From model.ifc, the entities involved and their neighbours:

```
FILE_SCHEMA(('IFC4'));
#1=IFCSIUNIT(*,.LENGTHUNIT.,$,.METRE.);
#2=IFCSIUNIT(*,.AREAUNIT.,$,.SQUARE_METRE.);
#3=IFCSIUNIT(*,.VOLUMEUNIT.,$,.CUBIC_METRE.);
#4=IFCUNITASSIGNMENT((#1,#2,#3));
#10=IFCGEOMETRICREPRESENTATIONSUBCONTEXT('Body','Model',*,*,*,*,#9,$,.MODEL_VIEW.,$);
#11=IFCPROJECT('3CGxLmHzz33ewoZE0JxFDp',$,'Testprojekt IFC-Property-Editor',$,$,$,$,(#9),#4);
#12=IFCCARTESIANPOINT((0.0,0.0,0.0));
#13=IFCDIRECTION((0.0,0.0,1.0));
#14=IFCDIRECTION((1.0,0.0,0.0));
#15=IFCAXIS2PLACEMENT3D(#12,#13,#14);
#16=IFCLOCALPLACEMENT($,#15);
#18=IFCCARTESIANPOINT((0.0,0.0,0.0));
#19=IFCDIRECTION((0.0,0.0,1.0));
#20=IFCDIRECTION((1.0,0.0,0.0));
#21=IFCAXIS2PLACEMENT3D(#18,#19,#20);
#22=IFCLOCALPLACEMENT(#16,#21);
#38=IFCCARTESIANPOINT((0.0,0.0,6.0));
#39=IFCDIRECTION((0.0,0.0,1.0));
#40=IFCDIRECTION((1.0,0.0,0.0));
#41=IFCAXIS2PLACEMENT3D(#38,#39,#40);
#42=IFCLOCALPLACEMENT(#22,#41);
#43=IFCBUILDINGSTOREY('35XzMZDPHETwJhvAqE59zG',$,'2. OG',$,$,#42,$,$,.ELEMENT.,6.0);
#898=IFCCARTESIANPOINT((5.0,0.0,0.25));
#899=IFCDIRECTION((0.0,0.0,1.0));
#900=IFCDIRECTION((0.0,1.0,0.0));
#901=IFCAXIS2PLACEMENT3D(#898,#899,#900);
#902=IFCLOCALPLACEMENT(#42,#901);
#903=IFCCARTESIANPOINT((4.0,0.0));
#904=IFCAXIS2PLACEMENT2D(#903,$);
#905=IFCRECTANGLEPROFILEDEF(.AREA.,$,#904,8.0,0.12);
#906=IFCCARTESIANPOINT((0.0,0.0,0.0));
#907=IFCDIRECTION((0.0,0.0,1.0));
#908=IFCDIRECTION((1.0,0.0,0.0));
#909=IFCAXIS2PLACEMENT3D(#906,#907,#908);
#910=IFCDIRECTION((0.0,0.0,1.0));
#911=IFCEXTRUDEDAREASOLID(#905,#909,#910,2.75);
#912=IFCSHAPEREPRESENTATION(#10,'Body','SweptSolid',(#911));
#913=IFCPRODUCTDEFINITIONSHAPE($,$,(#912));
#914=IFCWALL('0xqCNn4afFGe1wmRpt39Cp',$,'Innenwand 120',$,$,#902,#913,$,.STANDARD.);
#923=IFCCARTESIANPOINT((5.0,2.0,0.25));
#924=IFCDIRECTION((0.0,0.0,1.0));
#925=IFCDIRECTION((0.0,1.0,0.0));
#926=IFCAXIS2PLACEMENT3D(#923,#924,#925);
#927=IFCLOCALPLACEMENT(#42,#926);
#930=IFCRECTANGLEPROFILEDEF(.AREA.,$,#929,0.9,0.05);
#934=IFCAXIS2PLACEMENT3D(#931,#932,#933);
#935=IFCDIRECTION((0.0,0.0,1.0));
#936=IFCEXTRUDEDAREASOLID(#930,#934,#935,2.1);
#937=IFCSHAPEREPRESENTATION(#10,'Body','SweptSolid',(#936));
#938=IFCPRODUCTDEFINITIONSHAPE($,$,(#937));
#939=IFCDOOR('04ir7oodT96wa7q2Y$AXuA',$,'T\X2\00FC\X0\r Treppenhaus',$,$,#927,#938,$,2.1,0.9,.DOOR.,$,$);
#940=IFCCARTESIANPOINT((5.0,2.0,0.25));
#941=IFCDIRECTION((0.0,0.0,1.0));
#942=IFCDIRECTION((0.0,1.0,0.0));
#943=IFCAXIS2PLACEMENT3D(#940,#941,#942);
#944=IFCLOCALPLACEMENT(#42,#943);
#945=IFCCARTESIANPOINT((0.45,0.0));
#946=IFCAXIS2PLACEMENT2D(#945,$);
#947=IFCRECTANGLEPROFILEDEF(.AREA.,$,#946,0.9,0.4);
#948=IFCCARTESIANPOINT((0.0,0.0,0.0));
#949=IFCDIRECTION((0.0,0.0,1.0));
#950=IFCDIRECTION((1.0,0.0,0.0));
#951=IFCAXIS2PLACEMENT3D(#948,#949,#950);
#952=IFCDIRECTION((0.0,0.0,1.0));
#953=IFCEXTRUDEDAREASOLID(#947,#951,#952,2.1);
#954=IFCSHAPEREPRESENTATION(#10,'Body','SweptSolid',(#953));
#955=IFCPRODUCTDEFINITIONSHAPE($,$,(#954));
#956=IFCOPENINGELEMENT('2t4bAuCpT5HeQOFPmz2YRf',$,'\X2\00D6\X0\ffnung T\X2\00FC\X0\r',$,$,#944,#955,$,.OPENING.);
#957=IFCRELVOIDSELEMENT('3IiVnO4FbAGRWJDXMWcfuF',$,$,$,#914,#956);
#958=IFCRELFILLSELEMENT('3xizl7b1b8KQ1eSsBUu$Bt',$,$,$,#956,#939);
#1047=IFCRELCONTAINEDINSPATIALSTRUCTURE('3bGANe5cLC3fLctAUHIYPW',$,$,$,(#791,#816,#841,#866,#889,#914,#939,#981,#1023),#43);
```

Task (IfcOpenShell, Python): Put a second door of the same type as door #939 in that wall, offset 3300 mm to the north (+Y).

```python
import ifcopenshell
import ifcopenshell.api.feature
import ifcopenshell.api.geometry
import ifcopenshell.api.root
import ifcopenshell.geom
import ifcopenshell.util.element
import ifcopenshell.util.placement
import ifcopenshell.util.shape

model = ifcopenshell.open("model.ifc")
settings = ifcopenshell.geom.settings()


def volume(element):
    """Net volume in cubic metres, openings subtracted."""
    shape = ifcopenshell.geom.create_shape(settings, element)
    return ifcopenshell.util.shape.get_volume(shape.geometry)


door = model.by_guid("04ir7oodT96wa7q2Y$AXuA")
opening = door.FillsVoids[0].RelatingOpeningElement
wall = opening.VoidsElements[0].RelatingBuildingElement
before = volume(wall)
shift = ifcopenshell.util.placement.get_local_placement(wall.ObjectPlacement)[:3, 0] * 3.3

# copy_class copies the void relationship, type, container and properties, but no geometry.
new_opening = ifcopenshell.api.root.copy_class(model, product=opening)
new_opening.Representation = ifcopenshell.util.element.copy_deep(
    model, opening.Representation, exclude=["IfcGeometricRepresentationContext", "IfcRepresentationMap"]
)
new_door = ifcopenshell.api.root.copy_class(model, product=door)
new_door.Representation = ifcopenshell.util.element.copy_deep(
    model, door.Representation, exclude=["IfcGeometricRepresentationContext", "IfcRepresentationMap"]
)
ifcopenshell.api.feature.add_filling(model, opening=new_opening, element=new_door)

for old, new in ((opening, new_opening), (door, new_door)):
    matrix = ifcopenshell.util.placement.get_local_placement(old.ObjectPlacement)
    matrix[:3, 3] += shift
    ifcopenshell.api.geometry.edit_object_placement(model, product=new, matrix=matrix, is_si=False)

after = volume(wall)

print(f"wall volume {before:.3f} -> {after:.3f} m3")

model.write("model_edited.ifc")
```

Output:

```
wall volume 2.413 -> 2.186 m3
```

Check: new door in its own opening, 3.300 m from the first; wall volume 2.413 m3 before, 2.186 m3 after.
